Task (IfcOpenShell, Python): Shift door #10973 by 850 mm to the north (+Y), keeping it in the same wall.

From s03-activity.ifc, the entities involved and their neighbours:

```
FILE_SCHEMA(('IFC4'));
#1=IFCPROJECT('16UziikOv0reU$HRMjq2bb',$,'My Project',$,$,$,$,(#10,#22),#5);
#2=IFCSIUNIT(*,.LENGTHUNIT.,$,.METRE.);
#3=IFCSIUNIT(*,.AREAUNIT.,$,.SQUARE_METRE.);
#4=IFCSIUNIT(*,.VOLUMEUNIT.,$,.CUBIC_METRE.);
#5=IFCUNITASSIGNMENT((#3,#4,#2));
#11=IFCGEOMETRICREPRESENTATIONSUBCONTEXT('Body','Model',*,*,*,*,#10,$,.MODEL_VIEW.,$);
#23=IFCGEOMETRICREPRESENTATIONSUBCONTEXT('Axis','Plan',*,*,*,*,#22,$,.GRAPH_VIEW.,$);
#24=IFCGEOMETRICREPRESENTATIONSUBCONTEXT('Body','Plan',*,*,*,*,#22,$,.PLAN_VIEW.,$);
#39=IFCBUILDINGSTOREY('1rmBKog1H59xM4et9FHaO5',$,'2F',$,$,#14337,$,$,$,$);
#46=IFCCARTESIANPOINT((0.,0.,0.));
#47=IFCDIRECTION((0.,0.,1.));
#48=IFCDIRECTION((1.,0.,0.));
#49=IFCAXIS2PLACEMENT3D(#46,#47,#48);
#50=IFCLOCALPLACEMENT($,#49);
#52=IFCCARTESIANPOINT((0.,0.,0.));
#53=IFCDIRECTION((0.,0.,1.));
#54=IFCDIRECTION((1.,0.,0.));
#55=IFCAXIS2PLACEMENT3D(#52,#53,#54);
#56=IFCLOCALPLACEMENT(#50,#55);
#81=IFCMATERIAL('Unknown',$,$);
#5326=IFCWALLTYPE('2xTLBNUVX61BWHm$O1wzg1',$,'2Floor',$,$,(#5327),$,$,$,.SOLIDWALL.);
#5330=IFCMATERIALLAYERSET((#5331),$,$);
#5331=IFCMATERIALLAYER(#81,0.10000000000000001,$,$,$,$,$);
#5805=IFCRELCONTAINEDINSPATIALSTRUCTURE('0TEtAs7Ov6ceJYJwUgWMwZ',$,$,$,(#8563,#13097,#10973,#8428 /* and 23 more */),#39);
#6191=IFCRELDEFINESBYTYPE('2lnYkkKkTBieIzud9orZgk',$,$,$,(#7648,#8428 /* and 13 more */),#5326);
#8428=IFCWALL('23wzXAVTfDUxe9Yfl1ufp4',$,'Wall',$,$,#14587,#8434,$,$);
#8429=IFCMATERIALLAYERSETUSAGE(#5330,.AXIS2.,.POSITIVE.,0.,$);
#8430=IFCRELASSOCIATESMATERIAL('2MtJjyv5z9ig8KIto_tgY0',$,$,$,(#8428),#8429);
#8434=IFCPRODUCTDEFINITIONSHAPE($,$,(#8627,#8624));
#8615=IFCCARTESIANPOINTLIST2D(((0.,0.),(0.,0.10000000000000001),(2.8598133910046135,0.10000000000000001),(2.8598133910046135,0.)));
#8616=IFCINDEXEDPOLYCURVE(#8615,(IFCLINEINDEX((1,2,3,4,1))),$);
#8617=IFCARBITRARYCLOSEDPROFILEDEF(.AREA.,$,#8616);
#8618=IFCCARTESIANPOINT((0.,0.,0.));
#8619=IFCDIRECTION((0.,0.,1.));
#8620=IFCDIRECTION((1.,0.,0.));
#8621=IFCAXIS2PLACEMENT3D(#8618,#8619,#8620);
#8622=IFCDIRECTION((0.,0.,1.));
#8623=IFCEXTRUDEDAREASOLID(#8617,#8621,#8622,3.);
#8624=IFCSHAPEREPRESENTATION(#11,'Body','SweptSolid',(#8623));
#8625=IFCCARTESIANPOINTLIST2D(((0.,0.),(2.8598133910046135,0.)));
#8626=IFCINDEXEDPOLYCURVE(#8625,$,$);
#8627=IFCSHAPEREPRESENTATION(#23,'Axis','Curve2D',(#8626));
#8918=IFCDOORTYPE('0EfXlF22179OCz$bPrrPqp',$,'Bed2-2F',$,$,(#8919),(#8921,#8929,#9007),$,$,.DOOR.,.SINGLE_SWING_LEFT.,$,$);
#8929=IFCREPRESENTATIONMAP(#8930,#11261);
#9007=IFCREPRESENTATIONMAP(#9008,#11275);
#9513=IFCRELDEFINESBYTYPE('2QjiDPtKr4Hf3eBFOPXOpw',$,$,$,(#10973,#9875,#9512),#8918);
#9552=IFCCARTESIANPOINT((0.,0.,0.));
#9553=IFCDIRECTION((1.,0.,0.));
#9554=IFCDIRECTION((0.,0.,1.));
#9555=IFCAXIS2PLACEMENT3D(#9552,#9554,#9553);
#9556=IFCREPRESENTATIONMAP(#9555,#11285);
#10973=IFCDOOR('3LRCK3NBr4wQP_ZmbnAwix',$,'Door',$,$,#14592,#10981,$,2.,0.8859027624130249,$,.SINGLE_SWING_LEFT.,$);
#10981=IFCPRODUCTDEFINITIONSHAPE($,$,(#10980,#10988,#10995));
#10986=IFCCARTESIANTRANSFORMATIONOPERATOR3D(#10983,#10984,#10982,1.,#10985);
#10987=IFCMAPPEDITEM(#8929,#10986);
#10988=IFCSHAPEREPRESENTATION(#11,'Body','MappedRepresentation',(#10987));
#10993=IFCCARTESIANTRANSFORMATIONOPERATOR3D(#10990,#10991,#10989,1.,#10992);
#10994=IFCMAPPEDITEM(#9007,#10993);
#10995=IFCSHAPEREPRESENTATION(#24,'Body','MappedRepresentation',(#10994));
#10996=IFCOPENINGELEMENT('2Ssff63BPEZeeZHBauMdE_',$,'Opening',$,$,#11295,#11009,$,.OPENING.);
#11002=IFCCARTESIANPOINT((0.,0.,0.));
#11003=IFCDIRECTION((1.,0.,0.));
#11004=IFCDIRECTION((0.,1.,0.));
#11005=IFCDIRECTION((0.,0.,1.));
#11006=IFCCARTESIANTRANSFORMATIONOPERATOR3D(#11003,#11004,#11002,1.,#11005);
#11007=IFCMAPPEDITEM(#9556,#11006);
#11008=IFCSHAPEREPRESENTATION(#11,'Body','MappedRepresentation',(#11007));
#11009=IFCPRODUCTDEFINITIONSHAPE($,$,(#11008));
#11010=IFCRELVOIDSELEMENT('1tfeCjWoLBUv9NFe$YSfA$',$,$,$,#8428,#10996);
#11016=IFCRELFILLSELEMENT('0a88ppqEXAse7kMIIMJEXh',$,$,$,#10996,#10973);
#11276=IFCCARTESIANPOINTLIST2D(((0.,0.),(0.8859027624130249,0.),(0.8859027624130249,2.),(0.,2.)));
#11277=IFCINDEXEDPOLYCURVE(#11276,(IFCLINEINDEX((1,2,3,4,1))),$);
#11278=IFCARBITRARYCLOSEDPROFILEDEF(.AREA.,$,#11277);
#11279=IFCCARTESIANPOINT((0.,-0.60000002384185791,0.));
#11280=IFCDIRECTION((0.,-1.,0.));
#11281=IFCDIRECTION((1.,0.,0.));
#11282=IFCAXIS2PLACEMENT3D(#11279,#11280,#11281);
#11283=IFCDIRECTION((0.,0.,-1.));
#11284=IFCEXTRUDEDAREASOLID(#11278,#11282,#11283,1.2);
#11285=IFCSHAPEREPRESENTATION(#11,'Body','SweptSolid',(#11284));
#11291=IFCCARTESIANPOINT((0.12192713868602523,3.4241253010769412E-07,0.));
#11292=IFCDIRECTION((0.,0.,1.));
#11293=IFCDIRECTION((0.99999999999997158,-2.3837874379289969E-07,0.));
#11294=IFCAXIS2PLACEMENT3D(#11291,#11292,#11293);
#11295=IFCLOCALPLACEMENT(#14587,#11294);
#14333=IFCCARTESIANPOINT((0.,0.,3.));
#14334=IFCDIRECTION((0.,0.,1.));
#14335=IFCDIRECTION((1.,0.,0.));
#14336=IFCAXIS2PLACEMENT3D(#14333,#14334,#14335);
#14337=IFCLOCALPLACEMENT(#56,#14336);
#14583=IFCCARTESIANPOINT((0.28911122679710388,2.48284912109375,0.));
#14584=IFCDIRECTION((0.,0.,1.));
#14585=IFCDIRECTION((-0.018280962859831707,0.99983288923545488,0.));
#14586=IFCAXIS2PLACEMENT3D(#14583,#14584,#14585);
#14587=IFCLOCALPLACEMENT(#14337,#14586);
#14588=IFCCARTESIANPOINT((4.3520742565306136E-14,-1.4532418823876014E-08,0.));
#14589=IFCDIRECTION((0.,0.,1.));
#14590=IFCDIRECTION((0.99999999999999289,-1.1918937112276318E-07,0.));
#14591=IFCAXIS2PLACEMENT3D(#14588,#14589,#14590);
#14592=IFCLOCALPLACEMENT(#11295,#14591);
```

```python
import ifcopenshell
import ifcopenshell.api.geometry
import ifcopenshell.util.placement
import ifcopenshell.util.unit

model = ifcopenshell.open("s03-activity.ifc")
unit_scale = ifcopenshell.util.unit.calculate_unit_scale(model)

door = model.by_guid("3LRCK3NBr4wQP_ZmbnAwix")
opening = door.FillsVoids[0].RelatingOpeningElement
wall = opening.VoidsElements[0].RelatingBuildingElement

wall_matrix = ifcopenshell.util.placement.get_local_placement(wall.ObjectPlacement)
shift = wall_matrix[:3, 0] * 0.85 / unit_scale
before = ifcopenshell.util.placement.get_local_placement(door.ObjectPlacement)[:3, 3].copy()

# The door is placed relative to its opening, so it follows when the opening moves.
matrix = ifcopenshell.util.placement.get_local_placement(opening.ObjectPlacement)
matrix[:3, 3] += shift
ifcopenshell.api.geometry.edit_object_placement(
    model, product=opening, matrix=matrix, is_si=False, should_transform_children=True
)

after = ifcopenshell.util.placement.get_local_placement(door.ObjectPlacement)[:3, 3]
print("door moved by", (after - before).round(3) + 0.0)

model.write("s03-activity_rev.ifc")
```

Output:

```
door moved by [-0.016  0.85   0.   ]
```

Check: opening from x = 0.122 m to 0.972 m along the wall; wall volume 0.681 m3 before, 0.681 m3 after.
